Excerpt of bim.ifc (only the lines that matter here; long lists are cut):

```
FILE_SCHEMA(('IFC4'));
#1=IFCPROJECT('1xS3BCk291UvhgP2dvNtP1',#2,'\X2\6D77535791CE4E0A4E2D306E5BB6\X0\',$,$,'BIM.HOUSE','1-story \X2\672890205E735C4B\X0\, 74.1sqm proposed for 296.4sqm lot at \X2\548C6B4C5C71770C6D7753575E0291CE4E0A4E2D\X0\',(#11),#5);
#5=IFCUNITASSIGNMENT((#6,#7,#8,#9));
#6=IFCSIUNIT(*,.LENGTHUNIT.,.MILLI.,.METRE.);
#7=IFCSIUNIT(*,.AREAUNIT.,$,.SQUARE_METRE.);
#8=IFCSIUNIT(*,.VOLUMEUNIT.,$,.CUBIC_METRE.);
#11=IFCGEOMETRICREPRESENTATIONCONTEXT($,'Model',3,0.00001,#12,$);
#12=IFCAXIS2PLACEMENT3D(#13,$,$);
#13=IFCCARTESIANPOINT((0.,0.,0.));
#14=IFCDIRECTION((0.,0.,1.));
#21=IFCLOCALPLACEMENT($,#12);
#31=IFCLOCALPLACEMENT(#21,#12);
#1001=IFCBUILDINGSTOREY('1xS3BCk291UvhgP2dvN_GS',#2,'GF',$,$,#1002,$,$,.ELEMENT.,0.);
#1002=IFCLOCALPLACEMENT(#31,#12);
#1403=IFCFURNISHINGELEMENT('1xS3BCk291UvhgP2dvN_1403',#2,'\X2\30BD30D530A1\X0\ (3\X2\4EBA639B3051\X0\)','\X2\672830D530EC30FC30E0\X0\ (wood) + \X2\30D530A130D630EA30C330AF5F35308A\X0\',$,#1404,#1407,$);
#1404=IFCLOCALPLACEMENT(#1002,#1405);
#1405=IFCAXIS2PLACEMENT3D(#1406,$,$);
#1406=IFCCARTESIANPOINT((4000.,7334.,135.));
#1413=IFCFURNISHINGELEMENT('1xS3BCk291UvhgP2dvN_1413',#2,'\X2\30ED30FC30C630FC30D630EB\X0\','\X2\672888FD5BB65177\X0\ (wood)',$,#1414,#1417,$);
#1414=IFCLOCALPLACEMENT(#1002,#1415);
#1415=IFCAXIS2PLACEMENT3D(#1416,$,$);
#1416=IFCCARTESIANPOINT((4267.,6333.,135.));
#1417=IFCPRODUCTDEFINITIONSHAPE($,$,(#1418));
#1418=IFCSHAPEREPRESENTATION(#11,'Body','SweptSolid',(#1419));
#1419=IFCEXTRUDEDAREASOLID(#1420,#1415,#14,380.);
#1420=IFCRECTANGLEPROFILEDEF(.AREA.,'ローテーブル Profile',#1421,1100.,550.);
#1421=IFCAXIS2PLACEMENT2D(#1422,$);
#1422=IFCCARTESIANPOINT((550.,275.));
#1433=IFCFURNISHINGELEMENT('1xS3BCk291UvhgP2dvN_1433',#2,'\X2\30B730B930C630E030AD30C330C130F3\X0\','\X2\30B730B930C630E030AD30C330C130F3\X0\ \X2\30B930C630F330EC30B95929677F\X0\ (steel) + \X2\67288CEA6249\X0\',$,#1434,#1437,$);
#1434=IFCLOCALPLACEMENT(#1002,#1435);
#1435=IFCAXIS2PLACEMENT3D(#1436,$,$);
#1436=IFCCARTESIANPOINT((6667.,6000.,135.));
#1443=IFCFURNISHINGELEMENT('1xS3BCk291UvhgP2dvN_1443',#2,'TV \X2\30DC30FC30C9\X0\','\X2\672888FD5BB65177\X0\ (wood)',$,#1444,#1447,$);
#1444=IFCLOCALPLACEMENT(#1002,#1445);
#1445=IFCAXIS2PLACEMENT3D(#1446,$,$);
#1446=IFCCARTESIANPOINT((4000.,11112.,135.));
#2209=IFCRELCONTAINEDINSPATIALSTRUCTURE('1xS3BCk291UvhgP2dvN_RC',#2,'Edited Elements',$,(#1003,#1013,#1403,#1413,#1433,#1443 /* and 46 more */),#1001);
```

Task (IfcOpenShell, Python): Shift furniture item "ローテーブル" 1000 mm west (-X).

```python
import ifcopenshell
import ifcopenshell.api.geometry
import ifcopenshell.util.placement
import ifcopenshell.util.unit

model = ifcopenshell.open("bim.ifc")
unit_scale = ifcopenshell.util.unit.calculate_unit_scale(model)

item = model.by_guid("1xS3BCk291UvhgP2dvN_1413")
matrix = ifcopenshell.util.placement.get_local_placement(item.ObjectPlacement)
matrix[0, 3] -= 1 / unit_scale
ifcopenshell.api.geometry.edit_object_placement(model, product=item, matrix=matrix, is_si=False)

print(ifcopenshell.util.placement.get_local_placement(item.ObjectPlacement).round(3) + 0.0)

model.write("bim_v2.ifc")
```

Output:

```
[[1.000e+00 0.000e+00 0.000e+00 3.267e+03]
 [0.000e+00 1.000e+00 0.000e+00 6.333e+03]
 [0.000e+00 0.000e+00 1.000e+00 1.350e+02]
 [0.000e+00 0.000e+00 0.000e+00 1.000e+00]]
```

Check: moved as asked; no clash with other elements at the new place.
